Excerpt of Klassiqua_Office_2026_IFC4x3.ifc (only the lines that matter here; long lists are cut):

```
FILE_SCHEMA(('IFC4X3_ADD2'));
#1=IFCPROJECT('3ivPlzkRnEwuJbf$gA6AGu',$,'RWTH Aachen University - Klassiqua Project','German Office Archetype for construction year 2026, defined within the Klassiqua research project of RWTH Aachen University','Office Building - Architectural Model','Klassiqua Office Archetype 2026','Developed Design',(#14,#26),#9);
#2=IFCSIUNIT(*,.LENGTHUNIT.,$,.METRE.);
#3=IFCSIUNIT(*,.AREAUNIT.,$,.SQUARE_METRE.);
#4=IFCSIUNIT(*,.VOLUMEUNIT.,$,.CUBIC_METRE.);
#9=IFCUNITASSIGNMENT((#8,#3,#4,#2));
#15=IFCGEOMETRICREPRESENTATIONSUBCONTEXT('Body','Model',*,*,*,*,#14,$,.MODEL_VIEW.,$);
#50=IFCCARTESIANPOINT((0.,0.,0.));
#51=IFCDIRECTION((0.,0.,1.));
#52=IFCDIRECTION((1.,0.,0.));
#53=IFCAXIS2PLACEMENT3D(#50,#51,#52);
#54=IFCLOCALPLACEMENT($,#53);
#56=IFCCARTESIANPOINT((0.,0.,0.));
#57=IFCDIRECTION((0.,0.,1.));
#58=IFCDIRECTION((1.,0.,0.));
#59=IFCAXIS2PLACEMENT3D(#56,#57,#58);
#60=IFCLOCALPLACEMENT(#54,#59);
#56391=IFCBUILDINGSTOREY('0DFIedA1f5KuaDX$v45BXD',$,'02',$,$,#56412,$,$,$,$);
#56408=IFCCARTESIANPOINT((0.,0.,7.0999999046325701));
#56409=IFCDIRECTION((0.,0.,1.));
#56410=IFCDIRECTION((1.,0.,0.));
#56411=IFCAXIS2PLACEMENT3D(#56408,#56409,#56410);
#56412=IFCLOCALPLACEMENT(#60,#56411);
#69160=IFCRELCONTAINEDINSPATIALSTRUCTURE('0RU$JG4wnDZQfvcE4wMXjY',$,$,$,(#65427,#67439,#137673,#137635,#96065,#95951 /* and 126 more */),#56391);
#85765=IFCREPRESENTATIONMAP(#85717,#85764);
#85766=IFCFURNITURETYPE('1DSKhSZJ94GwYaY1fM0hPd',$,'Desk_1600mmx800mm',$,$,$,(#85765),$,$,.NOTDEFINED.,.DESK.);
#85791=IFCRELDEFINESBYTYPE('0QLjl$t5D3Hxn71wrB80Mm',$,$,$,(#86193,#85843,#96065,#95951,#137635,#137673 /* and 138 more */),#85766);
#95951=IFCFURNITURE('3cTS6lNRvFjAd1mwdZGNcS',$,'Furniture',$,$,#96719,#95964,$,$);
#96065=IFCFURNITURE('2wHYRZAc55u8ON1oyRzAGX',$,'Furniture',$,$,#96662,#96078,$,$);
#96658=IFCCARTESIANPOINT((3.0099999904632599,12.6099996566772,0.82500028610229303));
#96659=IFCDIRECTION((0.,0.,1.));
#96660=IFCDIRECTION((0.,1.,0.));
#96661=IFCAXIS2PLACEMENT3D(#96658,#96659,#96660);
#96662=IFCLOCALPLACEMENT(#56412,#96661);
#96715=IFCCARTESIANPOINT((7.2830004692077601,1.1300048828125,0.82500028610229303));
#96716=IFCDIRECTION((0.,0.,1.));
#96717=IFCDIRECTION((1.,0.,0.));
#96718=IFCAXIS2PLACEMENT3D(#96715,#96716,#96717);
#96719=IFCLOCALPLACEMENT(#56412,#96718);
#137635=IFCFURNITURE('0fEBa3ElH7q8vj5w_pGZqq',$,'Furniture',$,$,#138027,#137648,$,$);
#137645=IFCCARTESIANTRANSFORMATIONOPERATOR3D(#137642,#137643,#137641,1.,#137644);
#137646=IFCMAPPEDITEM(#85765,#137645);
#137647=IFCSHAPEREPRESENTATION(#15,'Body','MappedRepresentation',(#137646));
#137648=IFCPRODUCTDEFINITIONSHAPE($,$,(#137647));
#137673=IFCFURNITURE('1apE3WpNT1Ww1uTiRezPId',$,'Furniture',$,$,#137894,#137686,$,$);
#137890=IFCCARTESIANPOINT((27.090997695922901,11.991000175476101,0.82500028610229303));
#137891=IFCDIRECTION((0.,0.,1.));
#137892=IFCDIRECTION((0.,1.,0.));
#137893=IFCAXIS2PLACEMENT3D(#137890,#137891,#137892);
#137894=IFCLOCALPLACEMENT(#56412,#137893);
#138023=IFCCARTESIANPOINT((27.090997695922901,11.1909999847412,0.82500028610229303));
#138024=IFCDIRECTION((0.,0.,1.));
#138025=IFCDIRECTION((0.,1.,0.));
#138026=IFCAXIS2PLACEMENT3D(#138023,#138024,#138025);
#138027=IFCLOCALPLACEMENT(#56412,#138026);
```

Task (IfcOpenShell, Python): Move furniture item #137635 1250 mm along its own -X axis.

```python
import ifcopenshell
import ifcopenshell.api.geometry
import ifcopenshell.util.placement
import ifcopenshell.util.unit

model = ifcopenshell.open("Klassiqua_Office_2026_IFC4x3.ifc")
unit_scale = ifcopenshell.util.unit.calculate_unit_scale(model)

item = model.by_guid("0fEBa3ElH7q8vj5w_pGZqq")
matrix = ifcopenshell.util.placement.get_local_placement(item.ObjectPlacement)
matrix[:3, 3] -= matrix[:3, 0] * 1.25 / unit_scale
ifcopenshell.api.geometry.edit_object_placement(model, product=item, matrix=matrix, is_si=False)

print(ifcopenshell.util.placement.get_local_placement(item.ObjectPlacement).round(3) + 0.0)

model.write("Klassiqua_Office_2026_IFC4x3_updated.ifc")
```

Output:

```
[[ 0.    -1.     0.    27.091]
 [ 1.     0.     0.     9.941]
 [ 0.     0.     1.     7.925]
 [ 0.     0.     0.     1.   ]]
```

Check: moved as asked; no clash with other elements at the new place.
